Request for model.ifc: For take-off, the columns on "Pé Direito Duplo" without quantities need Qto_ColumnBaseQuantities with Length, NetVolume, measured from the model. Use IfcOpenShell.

First a look at what the model holds.

```python
import ifcopenshell
import ifcopenshell.util.element
import ifcopenshell.util.unit

model = ifcopenshell.open("model.ifc")
print(model.schema)
for unit_type in ("LENGTHUNIT", "AREAUNIT", "VOLUMEUNIT"):
    print(unit_type, ifcopenshell.util.unit.calculate_unit_scale(model, unit_type))
storey = next(s for s in model.by_type("IfcBuildingStorey") if s.Name == "Pé Direito Duplo")
columns = [e for e in ifcopenshell.util.element.get_decomposition(storey) if e.is_a("IfcColumn")]
for e in sorted(columns, key=lambda e: e.id()):
    print(e.id(), e.is_a(), e.Name, list(ifcopenshell.util.element.get_psets(e, qtos_only=True)), sep=" | ")
```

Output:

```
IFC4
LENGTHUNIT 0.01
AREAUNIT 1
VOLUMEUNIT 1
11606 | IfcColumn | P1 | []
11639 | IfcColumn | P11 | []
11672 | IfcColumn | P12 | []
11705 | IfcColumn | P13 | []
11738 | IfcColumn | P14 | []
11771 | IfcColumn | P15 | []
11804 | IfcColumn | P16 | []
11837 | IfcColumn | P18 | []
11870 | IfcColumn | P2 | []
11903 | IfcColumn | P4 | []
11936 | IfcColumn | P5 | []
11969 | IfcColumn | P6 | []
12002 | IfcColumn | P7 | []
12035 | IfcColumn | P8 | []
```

```python
import ifcopenshell
import ifcopenshell.api.pset
import ifcopenshell.geom
import ifcopenshell.util.element
import ifcopenshell.util.shape
import ifcopenshell.util.unit

model = ifcopenshell.open("model.ifc")
unit_scale = ifcopenshell.util.unit.calculate_unit_scale(model)
volume_scale = ifcopenshell.util.unit.calculate_unit_scale(model, "VOLUMEUNIT")
settings = ifcopenshell.geom.settings()

storey = next(s for s in model.by_type("IfcBuildingStorey") if s.Name == "Pé Direito Duplo")
columns = [e for e in ifcopenshell.util.element.get_decomposition(storey) if e.is_a("IfcColumn")]

for e in sorted(columns, key=lambda e: e.id()):
    if ifcopenshell.util.element.get_psets(e, qtos_only=True, should_inherit=False):
        continue
    # Geometry comes back in metres, in the element's own axes.
    shape = ifcopenshell.geom.create_shape(settings, e)
    values = {
        "Length": ifcopenshell.util.shape.get_z(shape.geometry) / unit_scale,
        "NetVolume": ifcopenshell.util.shape.get_volume(shape.geometry) / volume_scale,
    }
    qto = ifcopenshell.api.pset.add_qto(model, product=e, name="Qto_ColumnBaseQuantities")
    ifcopenshell.api.pset.edit_qto(model, qto=qto, properties=values)
    print(e.id(), {k: round(v, 3) for k, v in values.items()})

model.write("model_updated.ifc")
```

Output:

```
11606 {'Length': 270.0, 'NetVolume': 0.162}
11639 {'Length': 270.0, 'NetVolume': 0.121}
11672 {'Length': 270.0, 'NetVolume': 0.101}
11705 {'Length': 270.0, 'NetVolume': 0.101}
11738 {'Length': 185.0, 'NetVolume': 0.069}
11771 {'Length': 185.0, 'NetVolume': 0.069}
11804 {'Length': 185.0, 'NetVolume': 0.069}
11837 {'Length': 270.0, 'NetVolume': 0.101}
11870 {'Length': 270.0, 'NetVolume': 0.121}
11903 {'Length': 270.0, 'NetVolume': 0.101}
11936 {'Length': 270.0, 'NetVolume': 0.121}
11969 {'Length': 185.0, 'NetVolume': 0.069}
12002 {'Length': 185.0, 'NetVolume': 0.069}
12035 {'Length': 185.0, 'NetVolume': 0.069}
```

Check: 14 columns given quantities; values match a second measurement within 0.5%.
